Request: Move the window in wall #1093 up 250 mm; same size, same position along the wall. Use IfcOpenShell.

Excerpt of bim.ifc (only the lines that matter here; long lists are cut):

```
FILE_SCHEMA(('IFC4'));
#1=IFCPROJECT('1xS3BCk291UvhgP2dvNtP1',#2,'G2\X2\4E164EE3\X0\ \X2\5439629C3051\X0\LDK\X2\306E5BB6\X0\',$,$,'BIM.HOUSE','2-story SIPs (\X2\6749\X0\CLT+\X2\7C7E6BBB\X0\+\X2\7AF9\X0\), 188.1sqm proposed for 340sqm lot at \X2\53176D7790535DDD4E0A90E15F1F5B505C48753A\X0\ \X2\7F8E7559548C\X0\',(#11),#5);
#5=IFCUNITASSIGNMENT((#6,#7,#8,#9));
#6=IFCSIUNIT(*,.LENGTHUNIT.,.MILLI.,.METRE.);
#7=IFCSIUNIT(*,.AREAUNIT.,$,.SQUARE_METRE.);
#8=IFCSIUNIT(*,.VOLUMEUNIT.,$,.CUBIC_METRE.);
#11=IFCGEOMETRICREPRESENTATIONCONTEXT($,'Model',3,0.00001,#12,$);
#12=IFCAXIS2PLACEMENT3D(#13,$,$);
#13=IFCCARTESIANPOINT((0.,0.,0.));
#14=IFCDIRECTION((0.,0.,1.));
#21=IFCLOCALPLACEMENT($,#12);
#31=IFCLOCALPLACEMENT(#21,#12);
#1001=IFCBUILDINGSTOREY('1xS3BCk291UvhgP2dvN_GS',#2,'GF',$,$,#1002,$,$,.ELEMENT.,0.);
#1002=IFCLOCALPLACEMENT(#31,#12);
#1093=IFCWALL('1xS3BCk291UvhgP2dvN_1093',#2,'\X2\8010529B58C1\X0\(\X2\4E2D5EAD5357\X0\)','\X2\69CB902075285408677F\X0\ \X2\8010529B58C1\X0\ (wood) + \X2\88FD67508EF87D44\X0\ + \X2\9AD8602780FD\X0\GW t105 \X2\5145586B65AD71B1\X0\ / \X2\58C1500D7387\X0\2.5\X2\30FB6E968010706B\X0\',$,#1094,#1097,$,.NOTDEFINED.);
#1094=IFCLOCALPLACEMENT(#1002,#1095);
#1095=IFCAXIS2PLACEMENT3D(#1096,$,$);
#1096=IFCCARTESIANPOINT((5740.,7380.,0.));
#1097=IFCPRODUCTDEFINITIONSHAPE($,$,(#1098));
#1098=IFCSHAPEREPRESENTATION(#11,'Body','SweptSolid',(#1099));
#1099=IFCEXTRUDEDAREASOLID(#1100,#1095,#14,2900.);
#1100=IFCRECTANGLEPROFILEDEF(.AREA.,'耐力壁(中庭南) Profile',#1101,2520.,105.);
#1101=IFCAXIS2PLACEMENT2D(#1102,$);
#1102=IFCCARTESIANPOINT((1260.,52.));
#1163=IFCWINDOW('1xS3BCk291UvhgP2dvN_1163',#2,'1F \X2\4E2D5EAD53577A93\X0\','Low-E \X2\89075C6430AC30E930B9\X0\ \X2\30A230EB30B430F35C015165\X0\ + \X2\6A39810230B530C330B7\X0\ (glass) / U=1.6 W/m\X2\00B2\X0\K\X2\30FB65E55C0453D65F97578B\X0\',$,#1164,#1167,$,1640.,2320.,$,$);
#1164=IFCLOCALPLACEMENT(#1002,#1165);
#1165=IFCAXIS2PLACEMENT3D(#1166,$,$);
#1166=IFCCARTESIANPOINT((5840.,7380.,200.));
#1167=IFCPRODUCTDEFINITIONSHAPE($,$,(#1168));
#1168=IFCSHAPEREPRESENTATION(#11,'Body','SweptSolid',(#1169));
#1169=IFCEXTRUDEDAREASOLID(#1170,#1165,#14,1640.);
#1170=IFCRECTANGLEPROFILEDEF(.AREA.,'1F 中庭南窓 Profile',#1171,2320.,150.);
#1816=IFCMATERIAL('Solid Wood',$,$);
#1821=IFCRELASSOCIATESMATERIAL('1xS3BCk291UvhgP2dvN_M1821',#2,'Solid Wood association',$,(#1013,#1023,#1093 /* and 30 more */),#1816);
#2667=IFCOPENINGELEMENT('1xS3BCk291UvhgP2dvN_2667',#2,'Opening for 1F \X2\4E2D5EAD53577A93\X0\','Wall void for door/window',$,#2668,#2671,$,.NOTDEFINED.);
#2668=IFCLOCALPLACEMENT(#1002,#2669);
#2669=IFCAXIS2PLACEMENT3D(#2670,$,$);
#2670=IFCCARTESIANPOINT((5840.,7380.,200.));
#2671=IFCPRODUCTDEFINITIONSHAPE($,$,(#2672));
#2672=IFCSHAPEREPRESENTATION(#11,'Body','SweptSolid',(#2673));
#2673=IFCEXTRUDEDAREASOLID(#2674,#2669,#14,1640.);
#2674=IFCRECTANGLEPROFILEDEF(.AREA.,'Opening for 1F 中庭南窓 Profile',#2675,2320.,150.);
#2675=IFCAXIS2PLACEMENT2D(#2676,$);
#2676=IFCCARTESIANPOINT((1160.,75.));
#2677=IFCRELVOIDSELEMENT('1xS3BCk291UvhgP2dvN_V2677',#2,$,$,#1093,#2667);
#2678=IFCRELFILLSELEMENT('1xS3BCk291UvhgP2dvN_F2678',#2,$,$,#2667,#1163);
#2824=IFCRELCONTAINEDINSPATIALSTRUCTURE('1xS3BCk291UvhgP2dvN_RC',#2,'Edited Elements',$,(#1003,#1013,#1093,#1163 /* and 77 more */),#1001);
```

```python
import numpy as np
import ifcopenshell
import ifcopenshell.api.geometry
import ifcopenshell.util.placement
import ifcopenshell.util.unit

model = ifcopenshell.open("bim.ifc")
unit_scale = ifcopenshell.util.unit.calculate_unit_scale(model)

window = model.by_guid("1xS3BCk291UvhgP2dvN_1163")
opening = window.FillsVoids[0].RelatingOpeningElement
dz = 250.0

shift = np.array([0.0, 0.0, dz])
# The window is not placed relative to its opening, so move both.
for product in (opening, window):
    matrix = ifcopenshell.util.placement.get_local_placement(product.ObjectPlacement)
    matrix[:3, 3] += shift
    ifcopenshell.api.geometry.edit_object_placement(model, product=product, matrix=matrix, is_si=False)

print(f"moved by {dz * unit_scale:+.3f} m")

model.write("bim-out.ifc")
```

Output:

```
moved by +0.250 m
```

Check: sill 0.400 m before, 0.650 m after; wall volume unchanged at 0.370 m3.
